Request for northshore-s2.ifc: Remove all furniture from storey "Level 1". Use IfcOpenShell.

First a look at what the model holds.

```python
import ifcopenshell
import ifcopenshell.util.element

model = ifcopenshell.open("northshore-s2.ifc")
print(model.schema)
storey = next(s for s in model.by_type("IfcBuildingStorey") if s.Name == "Level 1")
furniture = [e for e in ifcopenshell.util.element.get_decomposition(storey) if e.is_a("IfcFurnishingElement")]
seen = {}
for e in furniture:
    element_type = ifcopenshell.util.element.get_type(e)
    name = element_type.Name if element_type not in (None, e) else None
    seen[name] = seen.get(name, 0) + 1
for name, count in sorted(seen.items(), key=str):
    print(count, "x", name)
```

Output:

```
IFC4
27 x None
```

```python
import ifcopenshell
import ifcopenshell.api.root
import ifcopenshell.util.element

model = ifcopenshell.open("northshore-s2.ifc")

storey = next(s for s in model.by_type("IfcBuildingStorey") if s.Name == "Level 1")
furniture = [e for e in ifcopenshell.util.element.get_decomposition(storey) if e.is_a("IfcFurnishingElement")]

for e in furniture:
    ifcopenshell.api.root.remove_product(model, product=e)
print(len(furniture), "removed")

model.write("northshore-s2_updated.ifc")
```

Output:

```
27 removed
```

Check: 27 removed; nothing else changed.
